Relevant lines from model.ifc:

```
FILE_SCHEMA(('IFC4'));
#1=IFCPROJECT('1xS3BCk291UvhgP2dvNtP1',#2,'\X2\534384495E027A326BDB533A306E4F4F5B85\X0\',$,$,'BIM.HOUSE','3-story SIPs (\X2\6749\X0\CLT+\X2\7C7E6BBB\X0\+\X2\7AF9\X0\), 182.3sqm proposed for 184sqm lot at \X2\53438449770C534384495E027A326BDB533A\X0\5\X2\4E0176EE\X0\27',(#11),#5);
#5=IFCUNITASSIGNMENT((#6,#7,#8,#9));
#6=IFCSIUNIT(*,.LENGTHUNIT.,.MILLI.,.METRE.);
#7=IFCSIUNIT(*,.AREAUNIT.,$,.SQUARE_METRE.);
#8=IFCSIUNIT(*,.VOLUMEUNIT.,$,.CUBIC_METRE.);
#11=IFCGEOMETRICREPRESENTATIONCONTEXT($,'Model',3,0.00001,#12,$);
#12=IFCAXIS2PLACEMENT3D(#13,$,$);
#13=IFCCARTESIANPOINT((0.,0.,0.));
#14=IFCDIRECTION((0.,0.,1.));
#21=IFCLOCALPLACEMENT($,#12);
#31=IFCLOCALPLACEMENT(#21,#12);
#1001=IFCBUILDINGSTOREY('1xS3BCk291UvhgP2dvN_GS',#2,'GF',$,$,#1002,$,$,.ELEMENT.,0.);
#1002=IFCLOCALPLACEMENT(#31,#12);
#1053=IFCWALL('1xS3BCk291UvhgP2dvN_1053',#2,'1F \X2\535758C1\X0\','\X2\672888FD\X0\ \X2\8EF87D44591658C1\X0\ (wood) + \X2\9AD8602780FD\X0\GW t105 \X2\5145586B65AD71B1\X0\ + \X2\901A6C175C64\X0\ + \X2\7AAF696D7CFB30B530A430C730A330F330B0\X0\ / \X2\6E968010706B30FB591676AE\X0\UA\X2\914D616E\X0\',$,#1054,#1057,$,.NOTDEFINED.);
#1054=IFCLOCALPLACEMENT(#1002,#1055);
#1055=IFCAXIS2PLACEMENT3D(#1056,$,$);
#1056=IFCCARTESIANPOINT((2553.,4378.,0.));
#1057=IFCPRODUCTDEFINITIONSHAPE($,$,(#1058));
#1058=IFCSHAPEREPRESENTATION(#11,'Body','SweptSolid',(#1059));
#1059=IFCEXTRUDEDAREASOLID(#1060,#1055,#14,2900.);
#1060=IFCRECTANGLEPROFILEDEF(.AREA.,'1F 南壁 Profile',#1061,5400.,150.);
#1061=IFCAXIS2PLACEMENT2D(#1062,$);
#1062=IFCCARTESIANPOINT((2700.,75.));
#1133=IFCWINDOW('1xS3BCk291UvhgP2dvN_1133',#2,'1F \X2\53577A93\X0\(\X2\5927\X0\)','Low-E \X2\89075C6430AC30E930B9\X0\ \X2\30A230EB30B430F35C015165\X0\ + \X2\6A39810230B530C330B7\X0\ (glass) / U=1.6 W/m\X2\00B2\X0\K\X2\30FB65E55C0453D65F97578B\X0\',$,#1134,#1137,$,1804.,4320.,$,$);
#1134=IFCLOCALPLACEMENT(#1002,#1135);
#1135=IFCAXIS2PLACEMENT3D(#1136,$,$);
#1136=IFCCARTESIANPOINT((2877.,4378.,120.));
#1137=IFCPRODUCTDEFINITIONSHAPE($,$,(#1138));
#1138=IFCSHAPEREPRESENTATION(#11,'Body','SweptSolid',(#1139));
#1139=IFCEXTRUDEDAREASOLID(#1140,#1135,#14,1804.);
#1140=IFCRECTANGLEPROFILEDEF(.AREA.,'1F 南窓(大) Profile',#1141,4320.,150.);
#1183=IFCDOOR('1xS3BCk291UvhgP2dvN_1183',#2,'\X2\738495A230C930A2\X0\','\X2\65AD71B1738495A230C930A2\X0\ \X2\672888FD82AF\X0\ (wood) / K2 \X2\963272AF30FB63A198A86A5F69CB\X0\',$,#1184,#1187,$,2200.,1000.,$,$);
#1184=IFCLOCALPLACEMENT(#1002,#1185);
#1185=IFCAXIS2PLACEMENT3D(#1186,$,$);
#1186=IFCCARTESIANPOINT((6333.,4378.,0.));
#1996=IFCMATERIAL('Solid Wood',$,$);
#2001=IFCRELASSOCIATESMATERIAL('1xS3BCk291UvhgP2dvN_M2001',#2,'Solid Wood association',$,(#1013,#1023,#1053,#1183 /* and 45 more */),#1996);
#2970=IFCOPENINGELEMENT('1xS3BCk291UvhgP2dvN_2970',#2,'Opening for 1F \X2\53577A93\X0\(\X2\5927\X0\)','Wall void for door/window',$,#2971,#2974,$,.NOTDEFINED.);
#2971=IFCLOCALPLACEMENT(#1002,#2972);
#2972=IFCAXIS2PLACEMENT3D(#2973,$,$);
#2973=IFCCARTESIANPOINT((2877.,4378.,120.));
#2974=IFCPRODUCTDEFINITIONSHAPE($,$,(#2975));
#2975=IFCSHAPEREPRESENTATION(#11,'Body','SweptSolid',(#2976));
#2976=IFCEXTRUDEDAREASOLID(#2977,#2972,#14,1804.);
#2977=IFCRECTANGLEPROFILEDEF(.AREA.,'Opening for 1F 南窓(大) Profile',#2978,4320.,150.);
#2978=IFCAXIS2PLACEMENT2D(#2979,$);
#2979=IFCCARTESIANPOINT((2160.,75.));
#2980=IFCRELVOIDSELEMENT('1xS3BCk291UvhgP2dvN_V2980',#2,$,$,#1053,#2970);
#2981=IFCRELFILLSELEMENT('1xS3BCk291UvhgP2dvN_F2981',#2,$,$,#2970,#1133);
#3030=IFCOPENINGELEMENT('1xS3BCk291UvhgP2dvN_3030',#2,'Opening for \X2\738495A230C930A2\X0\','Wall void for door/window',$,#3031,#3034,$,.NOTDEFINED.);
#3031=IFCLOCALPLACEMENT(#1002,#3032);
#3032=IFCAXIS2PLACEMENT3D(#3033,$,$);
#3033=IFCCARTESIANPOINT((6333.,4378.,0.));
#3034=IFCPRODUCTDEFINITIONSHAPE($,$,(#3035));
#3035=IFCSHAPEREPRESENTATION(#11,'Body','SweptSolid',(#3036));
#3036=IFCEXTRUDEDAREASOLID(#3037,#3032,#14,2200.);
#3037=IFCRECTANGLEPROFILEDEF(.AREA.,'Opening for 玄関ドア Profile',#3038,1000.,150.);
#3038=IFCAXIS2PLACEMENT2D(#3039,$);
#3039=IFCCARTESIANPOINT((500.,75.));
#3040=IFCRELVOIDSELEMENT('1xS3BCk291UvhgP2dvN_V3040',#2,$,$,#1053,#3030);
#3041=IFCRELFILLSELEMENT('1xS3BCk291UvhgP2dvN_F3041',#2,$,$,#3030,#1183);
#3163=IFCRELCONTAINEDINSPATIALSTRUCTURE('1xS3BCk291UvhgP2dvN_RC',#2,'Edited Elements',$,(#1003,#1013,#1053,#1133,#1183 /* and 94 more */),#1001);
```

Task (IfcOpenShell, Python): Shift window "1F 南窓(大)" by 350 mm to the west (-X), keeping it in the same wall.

```python
import ifcopenshell
import ifcopenshell.api.geometry
import ifcopenshell.util.placement
import ifcopenshell.util.unit

model = ifcopenshell.open("model.ifc")
unit_scale = ifcopenshell.util.unit.calculate_unit_scale(model)

window = model.by_guid("1xS3BCk291UvhgP2dvN_1133")
opening = window.FillsVoids[0].RelatingOpeningElement
wall = opening.VoidsElements[0].RelatingBuildingElement

wall_matrix = ifcopenshell.util.placement.get_local_placement(wall.ObjectPlacement)
shift = wall_matrix[:3, 0] * -0.35 / unit_scale
before = ifcopenshell.util.placement.get_local_placement(window.ObjectPlacement)[:3, 3].copy()

# The window is not placed relative to its opening, so move both.
for product in (opening, window):
    matrix = ifcopenshell.util.placement.get_local_placement(product.ObjectPlacement)
    matrix[:3, 3] += shift
    ifcopenshell.api.geometry.edit_object_placement(model, product=product, matrix=matrix, is_si=False)

after = ifcopenshell.util.placement.get_local_placement(window.ObjectPlacement)[:3, 3]
print("window moved by", (after - before).round(3) + 0.0)

model.write("model_edited.ifc")
```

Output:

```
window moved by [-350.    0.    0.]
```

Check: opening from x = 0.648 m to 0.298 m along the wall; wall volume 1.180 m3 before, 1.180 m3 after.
